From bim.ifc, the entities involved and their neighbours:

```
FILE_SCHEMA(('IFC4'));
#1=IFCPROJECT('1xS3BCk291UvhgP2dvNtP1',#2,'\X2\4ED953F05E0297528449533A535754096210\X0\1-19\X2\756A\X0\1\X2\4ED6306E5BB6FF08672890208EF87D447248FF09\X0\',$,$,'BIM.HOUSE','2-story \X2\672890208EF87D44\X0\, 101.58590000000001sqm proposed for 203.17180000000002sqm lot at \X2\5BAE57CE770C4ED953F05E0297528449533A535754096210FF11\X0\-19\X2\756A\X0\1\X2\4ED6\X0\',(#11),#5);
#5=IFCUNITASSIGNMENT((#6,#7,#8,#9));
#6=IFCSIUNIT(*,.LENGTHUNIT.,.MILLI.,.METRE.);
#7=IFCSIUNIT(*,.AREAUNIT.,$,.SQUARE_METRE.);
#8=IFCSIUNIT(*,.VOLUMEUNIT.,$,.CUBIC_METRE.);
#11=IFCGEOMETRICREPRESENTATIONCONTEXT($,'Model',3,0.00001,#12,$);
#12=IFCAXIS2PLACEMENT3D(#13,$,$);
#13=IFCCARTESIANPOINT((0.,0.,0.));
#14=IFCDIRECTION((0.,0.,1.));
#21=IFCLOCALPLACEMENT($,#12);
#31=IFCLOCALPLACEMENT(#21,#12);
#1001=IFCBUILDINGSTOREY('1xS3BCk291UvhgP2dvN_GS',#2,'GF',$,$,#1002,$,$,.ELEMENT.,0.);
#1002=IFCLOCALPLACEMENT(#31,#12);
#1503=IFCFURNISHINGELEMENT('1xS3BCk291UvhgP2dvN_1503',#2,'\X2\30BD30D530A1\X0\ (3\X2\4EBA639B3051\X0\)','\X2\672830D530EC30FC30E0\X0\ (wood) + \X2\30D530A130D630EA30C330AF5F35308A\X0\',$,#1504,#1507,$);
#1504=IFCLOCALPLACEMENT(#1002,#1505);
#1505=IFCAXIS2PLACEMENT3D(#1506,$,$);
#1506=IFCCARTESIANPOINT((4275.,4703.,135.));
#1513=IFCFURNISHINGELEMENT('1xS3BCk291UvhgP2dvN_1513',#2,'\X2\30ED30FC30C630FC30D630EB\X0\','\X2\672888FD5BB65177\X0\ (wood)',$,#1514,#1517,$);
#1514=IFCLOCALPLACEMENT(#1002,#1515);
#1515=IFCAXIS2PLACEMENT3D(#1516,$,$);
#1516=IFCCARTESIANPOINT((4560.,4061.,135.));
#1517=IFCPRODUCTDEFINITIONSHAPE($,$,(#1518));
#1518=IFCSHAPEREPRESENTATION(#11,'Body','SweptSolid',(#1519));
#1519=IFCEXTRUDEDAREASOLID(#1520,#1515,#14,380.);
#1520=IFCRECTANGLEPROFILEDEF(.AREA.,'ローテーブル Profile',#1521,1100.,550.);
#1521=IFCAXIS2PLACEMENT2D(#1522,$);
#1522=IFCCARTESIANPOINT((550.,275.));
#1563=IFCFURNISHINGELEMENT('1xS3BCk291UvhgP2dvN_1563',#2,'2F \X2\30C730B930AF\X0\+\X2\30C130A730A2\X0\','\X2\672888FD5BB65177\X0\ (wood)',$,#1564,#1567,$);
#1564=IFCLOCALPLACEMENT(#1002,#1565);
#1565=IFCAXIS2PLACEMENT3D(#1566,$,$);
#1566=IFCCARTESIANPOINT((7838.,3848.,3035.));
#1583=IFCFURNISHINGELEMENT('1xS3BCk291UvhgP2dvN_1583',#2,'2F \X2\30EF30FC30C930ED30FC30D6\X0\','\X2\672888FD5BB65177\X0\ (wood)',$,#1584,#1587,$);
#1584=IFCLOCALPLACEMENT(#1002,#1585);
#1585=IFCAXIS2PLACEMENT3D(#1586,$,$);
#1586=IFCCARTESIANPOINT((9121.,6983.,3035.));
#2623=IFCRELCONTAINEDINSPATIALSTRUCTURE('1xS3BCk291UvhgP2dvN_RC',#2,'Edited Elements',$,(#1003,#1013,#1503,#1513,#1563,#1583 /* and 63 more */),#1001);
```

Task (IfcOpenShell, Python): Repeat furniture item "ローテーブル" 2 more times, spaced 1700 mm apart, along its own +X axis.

```python
import ifcopenshell
import ifcopenshell.api.geometry
import ifcopenshell.api.root
import ifcopenshell.util.element
import ifcopenshell.util.placement

model = ifcopenshell.open("bim.ifc")


def reuse_history(source, copy):
    """copy_class also copies each property set's owner history, people and application; keep the originals."""
    for rel in copy.IsDefinedBy:
        if rel.is_a("IfcRelDefinesByProperties") and (history := rel.RelatingPropertyDefinition.OwnerHistory):
            rel.RelatingPropertyDefinition.OwnerHistory = source.OwnerHistory
            ifcopenshell.util.element.remove_deep2(model, history)


source = model.by_guid("1xS3BCk291UvhgP2dvN_1513")
base = ifcopenshell.util.placement.get_local_placement(source.ObjectPlacement)
step = base[:3, 0] * 1700.0

for i in range(1, 3):
    copy = ifcopenshell.api.root.copy_class(model, product=source)
    copy.Representation = ifcopenshell.util.element.copy_deep(
        model, source.Representation, exclude=["IfcGeometricRepresentationContext", "IfcRepresentationMap"]
    )
    reuse_history(source, copy)
    matrix = base.copy()
    matrix[:3, 3] += i * step
    print("added at", matrix[:3, 3].round(3) + 0.0)
    ifcopenshell.api.geometry.edit_object_placement(model, product=copy, matrix=matrix, is_si=False)

model.write("bim_v2.ifc")
```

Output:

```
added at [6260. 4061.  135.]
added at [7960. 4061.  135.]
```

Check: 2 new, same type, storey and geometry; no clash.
